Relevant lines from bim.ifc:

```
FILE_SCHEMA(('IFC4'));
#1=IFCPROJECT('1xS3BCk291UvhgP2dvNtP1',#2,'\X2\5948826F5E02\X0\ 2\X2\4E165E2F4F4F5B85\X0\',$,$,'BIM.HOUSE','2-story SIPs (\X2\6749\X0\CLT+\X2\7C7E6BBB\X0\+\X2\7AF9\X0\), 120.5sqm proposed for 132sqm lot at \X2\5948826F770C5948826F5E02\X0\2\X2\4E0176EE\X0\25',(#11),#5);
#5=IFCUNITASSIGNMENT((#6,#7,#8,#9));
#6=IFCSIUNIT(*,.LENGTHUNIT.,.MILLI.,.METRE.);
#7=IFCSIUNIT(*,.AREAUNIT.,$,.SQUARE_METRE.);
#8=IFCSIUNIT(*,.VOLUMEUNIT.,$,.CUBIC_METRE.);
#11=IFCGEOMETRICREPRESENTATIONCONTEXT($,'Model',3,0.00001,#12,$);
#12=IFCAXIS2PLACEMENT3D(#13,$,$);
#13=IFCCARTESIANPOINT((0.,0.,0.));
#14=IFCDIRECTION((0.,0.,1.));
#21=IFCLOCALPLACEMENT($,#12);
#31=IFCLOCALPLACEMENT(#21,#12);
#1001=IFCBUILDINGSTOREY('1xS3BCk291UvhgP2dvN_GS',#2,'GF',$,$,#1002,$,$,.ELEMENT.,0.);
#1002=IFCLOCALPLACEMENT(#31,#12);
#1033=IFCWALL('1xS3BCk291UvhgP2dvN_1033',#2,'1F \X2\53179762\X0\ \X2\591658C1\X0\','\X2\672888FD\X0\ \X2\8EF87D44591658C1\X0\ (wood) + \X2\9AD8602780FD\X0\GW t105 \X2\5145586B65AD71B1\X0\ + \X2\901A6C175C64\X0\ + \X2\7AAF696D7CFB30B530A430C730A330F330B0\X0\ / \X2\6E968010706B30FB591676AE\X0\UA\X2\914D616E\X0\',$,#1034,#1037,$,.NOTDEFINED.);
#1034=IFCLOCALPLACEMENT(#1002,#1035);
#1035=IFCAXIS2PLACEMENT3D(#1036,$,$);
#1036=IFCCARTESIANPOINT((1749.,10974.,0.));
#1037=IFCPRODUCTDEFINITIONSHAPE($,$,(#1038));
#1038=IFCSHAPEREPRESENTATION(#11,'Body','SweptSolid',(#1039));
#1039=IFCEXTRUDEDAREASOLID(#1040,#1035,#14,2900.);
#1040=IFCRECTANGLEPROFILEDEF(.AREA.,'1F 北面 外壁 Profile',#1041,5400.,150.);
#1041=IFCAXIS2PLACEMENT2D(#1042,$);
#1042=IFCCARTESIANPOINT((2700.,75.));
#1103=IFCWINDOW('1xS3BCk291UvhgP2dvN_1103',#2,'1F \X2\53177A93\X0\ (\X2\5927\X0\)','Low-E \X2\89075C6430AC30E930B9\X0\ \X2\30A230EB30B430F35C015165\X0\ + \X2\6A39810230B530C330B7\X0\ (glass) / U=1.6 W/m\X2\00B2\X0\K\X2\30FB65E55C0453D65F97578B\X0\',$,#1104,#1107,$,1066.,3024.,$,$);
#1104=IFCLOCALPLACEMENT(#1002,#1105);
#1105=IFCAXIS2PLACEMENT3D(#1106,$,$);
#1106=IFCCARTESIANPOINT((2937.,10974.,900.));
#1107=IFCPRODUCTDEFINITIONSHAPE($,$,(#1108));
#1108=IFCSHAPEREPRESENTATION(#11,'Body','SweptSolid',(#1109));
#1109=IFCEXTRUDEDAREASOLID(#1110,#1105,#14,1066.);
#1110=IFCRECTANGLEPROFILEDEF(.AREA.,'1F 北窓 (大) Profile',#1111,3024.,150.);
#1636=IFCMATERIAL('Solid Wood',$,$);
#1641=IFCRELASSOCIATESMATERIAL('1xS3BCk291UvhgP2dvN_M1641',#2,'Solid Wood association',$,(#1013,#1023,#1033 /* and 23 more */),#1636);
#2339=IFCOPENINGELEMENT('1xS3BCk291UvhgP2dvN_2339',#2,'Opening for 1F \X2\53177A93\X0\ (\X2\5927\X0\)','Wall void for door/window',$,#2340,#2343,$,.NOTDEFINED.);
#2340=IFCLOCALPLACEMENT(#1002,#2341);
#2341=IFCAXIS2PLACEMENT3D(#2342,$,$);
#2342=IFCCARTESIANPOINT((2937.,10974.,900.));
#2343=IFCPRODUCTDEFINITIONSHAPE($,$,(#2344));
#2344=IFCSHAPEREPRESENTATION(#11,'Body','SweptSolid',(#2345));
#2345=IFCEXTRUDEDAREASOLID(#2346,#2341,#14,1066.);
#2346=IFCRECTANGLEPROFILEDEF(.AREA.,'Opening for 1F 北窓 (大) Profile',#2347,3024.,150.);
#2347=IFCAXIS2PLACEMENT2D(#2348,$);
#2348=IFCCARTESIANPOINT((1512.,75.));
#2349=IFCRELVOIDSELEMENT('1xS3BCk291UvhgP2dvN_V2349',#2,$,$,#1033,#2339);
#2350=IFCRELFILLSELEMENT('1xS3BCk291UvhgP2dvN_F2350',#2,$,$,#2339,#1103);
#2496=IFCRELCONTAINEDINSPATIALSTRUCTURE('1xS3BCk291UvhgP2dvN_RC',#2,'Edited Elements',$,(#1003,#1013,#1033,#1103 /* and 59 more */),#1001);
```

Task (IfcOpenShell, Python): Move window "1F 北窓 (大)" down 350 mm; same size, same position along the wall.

```python
import numpy as np
import ifcopenshell
import ifcopenshell.api.geometry
import ifcopenshell.util.placement
import ifcopenshell.util.unit

model = ifcopenshell.open("bim.ifc")
unit_scale = ifcopenshell.util.unit.calculate_unit_scale(model)

window = model.by_id(1103)
opening = window.FillsVoids[0].RelatingOpeningElement
dz = -350.0

shift = np.array([0.0, 0.0, dz])
# The window is not placed relative to its opening, so move both.
for product in (opening, window):
    matrix = ifcopenshell.util.placement.get_local_placement(product.ObjectPlacement)
    matrix[:3, 3] += shift
    ifcopenshell.api.geometry.edit_object_placement(model, product=product, matrix=matrix, is_si=False)

print(f"moved by {dz * unit_scale:+.3f} m")

model.write("bim_rev.ifc")
```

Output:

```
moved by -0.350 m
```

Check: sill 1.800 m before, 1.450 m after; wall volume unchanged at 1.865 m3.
